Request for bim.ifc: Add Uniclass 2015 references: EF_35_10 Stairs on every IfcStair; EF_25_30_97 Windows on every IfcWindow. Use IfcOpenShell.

First a look at what the model holds.

```python
import ifcopenshell

model = ifcopenshell.open("bim.ifc")
print(model.schema)
print("classifications:", [c.Name for c in model.by_type("IfcClassification")])
for ifc_class in ("IfcDoor", "IfcRoof", "IfcStair", "IfcWall", "IfcWindow"):
    print(ifc_class, len(model.by_type(ifc_class)))
```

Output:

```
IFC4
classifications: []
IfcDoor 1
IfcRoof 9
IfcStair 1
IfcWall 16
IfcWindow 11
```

```python
import ifcopenshell
import ifcopenshell.api.classification

model = ifcopenshell.open("bim.ifc")

system = ifcopenshell.api.classification.add_classification(model, classification="Uniclass 2015")

codes = {
    "IfcStair": ("EF_35_10", "Stairs"),
    "IfcWindow": ("EF_25_30_97", "Windows"),
}
for ifc_class, (code, name) in codes.items():
    products = model.by_type(ifc_class)
    ifcopenshell.api.classification.add_reference(
        model, products=products, classification=system, identification=code, name=name
    )
    print(code, len(products))

model.write("bim_edited.ifc")
```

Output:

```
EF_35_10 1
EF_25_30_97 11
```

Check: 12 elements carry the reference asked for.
